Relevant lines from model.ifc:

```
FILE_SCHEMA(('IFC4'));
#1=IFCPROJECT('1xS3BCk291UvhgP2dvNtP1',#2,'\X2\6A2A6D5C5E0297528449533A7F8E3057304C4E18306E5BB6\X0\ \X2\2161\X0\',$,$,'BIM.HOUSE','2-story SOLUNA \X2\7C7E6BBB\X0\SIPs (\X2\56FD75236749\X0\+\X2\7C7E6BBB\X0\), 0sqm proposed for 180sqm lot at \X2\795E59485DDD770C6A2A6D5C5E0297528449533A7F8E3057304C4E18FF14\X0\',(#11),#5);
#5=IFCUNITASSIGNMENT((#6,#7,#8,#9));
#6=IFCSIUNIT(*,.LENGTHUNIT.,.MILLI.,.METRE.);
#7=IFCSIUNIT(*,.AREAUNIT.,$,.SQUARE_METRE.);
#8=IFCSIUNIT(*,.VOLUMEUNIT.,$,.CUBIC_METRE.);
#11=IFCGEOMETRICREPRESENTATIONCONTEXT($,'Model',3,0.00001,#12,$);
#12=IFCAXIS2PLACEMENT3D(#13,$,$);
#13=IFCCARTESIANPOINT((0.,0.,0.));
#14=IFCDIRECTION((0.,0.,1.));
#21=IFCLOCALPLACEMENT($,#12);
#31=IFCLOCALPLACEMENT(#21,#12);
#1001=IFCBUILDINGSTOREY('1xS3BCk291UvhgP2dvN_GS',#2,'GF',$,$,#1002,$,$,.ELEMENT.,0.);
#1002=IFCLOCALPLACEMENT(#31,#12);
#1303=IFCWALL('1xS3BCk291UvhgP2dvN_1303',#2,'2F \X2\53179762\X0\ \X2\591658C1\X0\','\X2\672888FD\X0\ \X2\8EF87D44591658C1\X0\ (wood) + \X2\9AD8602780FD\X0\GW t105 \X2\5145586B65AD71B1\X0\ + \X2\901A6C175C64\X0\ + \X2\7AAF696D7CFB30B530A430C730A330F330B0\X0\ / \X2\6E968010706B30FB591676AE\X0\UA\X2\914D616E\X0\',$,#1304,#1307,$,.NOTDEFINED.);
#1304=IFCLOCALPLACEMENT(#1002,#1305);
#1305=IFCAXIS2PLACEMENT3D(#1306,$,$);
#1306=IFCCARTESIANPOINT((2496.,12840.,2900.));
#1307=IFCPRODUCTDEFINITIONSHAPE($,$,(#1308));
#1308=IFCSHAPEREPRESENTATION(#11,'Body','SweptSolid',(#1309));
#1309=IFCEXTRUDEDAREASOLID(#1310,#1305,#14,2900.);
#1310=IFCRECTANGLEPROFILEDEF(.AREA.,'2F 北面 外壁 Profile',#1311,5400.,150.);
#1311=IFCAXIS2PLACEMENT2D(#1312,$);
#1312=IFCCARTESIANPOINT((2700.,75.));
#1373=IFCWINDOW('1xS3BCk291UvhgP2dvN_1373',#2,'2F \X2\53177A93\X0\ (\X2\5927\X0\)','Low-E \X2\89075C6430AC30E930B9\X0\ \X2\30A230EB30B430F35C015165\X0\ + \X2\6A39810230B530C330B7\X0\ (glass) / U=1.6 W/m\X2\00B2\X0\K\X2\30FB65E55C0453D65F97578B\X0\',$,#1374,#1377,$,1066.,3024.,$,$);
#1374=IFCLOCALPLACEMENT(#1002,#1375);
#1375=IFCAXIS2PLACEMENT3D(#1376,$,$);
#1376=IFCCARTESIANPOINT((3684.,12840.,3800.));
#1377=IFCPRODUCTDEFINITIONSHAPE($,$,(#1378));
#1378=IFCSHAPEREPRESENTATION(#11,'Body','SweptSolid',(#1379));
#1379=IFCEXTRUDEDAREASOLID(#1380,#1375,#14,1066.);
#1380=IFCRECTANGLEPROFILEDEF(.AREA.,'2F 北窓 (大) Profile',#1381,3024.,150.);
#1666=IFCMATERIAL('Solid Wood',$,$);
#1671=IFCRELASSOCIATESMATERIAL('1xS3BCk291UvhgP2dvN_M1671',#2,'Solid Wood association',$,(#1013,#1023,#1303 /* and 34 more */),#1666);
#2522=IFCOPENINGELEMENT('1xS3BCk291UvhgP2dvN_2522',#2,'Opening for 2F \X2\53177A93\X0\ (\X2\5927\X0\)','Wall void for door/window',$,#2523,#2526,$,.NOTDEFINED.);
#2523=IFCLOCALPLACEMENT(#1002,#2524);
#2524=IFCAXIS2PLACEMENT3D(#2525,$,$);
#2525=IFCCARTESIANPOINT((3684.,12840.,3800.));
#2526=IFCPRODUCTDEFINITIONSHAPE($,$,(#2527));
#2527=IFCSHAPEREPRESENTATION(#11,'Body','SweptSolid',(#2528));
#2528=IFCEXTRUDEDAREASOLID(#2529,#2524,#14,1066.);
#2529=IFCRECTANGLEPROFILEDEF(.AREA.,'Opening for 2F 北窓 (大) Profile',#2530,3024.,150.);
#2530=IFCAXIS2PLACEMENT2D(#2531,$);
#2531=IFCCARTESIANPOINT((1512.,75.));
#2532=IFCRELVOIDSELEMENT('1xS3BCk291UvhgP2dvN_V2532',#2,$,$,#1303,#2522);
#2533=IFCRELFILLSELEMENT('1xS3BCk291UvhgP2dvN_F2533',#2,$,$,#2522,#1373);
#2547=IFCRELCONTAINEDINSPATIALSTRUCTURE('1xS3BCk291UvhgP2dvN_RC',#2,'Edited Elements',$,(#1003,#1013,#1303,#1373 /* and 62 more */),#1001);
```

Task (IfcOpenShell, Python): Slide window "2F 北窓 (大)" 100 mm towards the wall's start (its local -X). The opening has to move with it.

```python
import ifcopenshell
import ifcopenshell.api.geometry
import ifcopenshell.util.placement

model = ifcopenshell.open("model.ifc")

window = model.by_guid("1xS3BCk291UvhgP2dvN_1373")
opening = window.FillsVoids[0].RelatingOpeningElement
wall = opening.VoidsElements[0].RelatingBuildingElement

wall_matrix = ifcopenshell.util.placement.get_local_placement(wall.ObjectPlacement)
shift = wall_matrix[:3, 0] * -100.0
before = ifcopenshell.util.placement.get_local_placement(window.ObjectPlacement)[:3, 3].copy()

# The window is not placed relative to its opening, so move both.
for product in (opening, window):
    matrix = ifcopenshell.util.placement.get_local_placement(product.ObjectPlacement)
    matrix[:3, 3] += shift
    ifcopenshell.api.geometry.edit_object_placement(model, product=product, matrix=matrix, is_si=False)

after = ifcopenshell.util.placement.get_local_placement(window.ObjectPlacement)[:3, 3]
print("window moved by", (after - before).round(3) + 0.0)

model.write("model_rev.ifc")
```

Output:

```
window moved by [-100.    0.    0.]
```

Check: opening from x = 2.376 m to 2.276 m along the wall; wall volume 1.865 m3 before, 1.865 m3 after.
